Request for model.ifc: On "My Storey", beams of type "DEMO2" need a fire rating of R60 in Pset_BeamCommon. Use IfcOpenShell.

First a look at what the model holds.

```python
import ifcopenshell
import ifcopenshell.util.element

model = ifcopenshell.open("model.ifc")
print(model.schema)
storey = next(s for s in model.by_type("IfcBuildingStorey") if s.Name == "My Storey")
beams = [e for e in ifcopenshell.util.element.get_decomposition(storey) if e.is_a("IfcBeam")]
seen = {}
for e in beams:
    element_type = ifcopenshell.util.element.get_type(e)
    key = (element_type.Name if element_type != e and element_type else None, ifcopenshell.util.element.get_pset(e, "Pset_BeamCommon", "FireRating"))
    seen[key] = seen.get(key, 0) + 1
for (name, value), count in sorted(seen.items(), key=str):
    print(count, "x", name, "|", value)
```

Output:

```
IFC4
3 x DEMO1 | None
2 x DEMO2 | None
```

```python
import ifcopenshell
import ifcopenshell.api.pset
import ifcopenshell.util.element

model = ifcopenshell.open("model.ifc")

storey = next(s for s in model.by_type("IfcBuildingStorey") if s.Name == "My Storey")
beams = [e for e in ifcopenshell.util.element.get_decomposition(storey) if e.is_a("IfcBeam")]

count = 0
for e in beams:
    element_type = ifcopenshell.util.element.get_type(e)
    if element_type in (None, e) or element_type.Name != "DEMO2":
        continue
    # add_pset returns the element's existing set when there is one.
    pset = ifcopenshell.api.pset.add_pset(model, product=e, name="Pset_BeamCommon")
    ifcopenshell.api.pset.edit_pset(model, pset=pset, properties={"FireRating": "R60"})
    count += 1

print(count, "beams updated")

model.write("model_v2.ifc")
```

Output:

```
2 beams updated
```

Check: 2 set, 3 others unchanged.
